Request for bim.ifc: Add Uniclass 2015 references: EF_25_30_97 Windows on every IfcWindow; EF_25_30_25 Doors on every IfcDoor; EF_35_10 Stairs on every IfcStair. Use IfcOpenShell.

First a look at what the model holds.

```python
import ifcopenshell

model = ifcopenshell.open("bim.ifc")
print(model.schema)
print("classifications:", [c.Name for c in model.by_type("IfcClassification")])
for ifc_class in ("IfcDoor", "IfcRoof", "IfcStair", "IfcWall", "IfcWindow"):
    print(ifc_class, len(model.by_type(ifc_class)))
```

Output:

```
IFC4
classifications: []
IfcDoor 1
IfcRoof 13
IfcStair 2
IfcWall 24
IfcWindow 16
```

```python
import ifcopenshell
import ifcopenshell.api.classification

model = ifcopenshell.open("bim.ifc")

system = ifcopenshell.api.classification.add_classification(model, classification="Uniclass 2015")

codes = {
    "IfcWindow": ("EF_25_30_97", "Windows"),
    "IfcDoor": ("EF_25_30_25", "Doors"),
    "IfcStair": ("EF_35_10", "Stairs"),
}
for ifc_class, (code, name) in codes.items():
    products = model.by_type(ifc_class)
    ifcopenshell.api.classification.add_reference(
        model, products=products, classification=system, identification=code, name=name
    )
    print(code, len(products))

model.write("bim_edited.ifc")
```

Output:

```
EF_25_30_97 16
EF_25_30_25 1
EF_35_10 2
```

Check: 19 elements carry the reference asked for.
